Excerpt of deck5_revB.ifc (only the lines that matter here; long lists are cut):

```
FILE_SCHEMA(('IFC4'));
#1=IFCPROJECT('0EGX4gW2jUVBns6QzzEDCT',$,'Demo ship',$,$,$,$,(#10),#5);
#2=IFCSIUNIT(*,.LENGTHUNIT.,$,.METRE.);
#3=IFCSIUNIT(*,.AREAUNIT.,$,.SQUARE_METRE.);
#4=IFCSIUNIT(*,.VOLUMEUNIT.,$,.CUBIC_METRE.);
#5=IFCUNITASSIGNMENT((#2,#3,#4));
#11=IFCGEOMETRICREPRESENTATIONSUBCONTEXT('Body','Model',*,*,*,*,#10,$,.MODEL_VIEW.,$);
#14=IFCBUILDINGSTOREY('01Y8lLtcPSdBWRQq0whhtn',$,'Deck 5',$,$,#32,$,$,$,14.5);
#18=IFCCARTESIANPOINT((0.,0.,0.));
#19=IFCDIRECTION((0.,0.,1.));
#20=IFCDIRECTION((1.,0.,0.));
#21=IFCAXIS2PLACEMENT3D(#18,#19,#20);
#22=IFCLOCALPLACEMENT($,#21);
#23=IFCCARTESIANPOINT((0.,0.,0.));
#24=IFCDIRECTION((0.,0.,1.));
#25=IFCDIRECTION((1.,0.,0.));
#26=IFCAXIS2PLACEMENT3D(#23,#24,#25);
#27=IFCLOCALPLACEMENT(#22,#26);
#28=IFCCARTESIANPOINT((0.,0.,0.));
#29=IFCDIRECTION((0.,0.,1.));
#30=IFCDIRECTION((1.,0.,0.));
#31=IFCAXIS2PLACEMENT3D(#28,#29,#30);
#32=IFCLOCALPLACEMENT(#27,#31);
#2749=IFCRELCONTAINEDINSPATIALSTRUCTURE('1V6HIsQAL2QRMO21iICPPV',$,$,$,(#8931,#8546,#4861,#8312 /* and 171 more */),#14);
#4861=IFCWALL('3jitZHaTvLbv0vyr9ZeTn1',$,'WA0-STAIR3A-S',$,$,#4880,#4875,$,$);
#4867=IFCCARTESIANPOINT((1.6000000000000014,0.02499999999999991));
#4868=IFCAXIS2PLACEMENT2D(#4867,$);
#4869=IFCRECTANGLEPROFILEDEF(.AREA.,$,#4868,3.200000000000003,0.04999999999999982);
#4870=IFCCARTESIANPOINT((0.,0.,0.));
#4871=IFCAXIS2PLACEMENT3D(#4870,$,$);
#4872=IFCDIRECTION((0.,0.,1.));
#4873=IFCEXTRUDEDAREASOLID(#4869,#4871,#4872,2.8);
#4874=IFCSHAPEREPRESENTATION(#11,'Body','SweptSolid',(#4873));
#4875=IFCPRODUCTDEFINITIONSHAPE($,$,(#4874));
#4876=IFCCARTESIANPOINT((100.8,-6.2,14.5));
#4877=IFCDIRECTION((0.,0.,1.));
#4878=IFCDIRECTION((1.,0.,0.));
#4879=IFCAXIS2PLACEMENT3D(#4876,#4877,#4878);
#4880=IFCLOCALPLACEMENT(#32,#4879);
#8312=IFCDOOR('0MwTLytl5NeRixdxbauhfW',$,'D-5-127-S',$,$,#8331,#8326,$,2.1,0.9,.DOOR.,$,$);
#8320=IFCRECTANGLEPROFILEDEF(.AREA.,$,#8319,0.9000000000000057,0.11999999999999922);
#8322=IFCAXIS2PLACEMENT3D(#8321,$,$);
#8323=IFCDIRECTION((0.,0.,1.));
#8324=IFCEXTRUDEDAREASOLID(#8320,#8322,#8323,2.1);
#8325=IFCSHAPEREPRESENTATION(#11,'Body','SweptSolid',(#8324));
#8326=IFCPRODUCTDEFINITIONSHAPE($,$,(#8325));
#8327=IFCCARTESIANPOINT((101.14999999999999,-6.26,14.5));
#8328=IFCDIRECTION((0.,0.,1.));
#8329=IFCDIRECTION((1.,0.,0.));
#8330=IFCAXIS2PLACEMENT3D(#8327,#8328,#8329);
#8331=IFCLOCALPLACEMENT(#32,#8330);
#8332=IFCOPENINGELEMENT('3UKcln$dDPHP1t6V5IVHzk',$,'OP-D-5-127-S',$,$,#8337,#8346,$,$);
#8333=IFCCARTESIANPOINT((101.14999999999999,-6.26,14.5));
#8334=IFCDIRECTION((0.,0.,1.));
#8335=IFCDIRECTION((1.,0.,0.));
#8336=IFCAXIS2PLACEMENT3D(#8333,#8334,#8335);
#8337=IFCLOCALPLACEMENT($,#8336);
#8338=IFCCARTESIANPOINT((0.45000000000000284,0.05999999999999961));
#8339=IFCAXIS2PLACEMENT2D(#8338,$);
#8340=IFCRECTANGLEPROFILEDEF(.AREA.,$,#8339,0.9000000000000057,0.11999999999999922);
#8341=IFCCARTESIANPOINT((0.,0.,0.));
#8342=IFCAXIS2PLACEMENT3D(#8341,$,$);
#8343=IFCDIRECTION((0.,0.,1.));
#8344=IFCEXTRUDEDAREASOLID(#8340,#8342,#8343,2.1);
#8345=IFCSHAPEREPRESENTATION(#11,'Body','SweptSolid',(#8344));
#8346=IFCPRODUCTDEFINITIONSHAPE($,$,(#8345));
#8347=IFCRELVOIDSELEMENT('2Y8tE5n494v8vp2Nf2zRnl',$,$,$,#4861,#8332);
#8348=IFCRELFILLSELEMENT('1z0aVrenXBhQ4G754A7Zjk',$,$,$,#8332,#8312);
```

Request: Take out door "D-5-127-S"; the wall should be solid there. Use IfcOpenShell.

```python
import ifcopenshell
import ifcopenshell.api.feature
import ifcopenshell.api.root
import ifcopenshell.geom
import ifcopenshell.util.shape

model = ifcopenshell.open("deck5_revB.ifc")
settings = ifcopenshell.geom.settings()


def volume(element):
    """Net volume in cubic metres, openings subtracted."""
    shape = ifcopenshell.geom.create_shape(settings, element)
    return ifcopenshell.util.shape.get_volume(shape.geometry)


door = model.by_id(8312)
opening = door.FillsVoids[0].RelatingOpeningElement
wall = opening.VoidsElements[0].RelatingBuildingElement
before = volume(wall)

ifcopenshell.api.root.remove_product(model, product=door)
ifcopenshell.api.feature.remove_feature(model, feature=opening)

after = volume(wall)

print(f"wall volume {before:.3f} -> {after:.3f} m3")

model.write("deck5_revB_updated.ifc")
```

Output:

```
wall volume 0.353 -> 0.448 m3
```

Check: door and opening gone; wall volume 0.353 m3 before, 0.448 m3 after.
